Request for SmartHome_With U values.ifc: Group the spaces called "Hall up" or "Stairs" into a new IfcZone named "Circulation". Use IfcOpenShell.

First a look at what the model holds.

```python
import ifcopenshell

model = ifcopenshell.open("SmartHome_With U values.ifc")
print(model.schema)
seen = {}
for space in model.by_type("IfcSpace"):
    seen[space.LongName] = seen.get(space.LongName, 0) + 1
for name, count in sorted(seen.items(), key=str):
    print(count, "x", name)
print("zones:", [z.Name for z in model.by_type("IfcZone")][:20])
```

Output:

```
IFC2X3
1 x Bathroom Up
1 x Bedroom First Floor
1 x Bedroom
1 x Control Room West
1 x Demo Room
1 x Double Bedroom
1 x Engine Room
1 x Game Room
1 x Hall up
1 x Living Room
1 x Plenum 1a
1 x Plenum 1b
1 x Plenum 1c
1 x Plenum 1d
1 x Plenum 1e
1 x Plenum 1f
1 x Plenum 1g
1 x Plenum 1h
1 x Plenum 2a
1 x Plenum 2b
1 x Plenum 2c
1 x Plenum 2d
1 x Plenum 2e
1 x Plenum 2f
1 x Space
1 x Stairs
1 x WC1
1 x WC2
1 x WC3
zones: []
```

```python
import ifcopenshell
import ifcopenshell.api.group
import ifcopenshell.api.root

model = ifcopenshell.open("SmartHome_With U values.ifc")

names = {"Hall up", "Stairs"}
spaces = [s for s in model.by_type("IfcSpace") if s.LongName in names]

zone = ifcopenshell.api.root.create_entity(model, ifc_class="IfcZone", name="Circulation")
ifcopenshell.api.group.assign_group(model, products=spaces, group=zone)
print(len(spaces), "spaces in", zone.Name)

model.write("SmartHome_With U values_updated.ifc")
```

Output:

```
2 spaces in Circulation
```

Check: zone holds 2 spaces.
